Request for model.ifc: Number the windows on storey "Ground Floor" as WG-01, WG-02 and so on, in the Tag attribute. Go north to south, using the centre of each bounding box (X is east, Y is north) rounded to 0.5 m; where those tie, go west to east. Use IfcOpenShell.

First a look at what the model holds.

```python
import ifcopenshell
import ifcopenshell.util.element
import ifcopenshell.util.placement

model = ifcopenshell.open("model.ifc")
print(model.schema)
storey = next(s for s in model.by_type("IfcBuildingStorey") if s.Name == "Ground Floor")
windows = [e for e in ifcopenshell.util.element.get_decomposition(storey) if e.is_a("IfcWindow")]
for e in sorted(windows, key=lambda e: e.id()):
    origin = ifcopenshell.util.placement.get_local_placement(e.ObjectPlacement)[:3, 3]
    print(e.id(), e.Tag, e.Name, origin.round(2) + 0.0, sep=" | ")
```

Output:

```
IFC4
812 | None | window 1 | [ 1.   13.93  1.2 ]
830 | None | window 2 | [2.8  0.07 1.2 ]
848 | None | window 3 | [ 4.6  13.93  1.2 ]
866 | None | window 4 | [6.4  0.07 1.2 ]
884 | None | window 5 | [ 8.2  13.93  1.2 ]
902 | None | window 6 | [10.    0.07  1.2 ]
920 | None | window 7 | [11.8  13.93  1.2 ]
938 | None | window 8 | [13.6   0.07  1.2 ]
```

```python
import ifcopenshell
import ifcopenshell.geom
import ifcopenshell.util.element
import ifcopenshell.util.shape

model = ifcopenshell.open("model.ifc")
settings = ifcopenshell.geom.settings()
settings.set("use-world-coords", True)


def centre(element):
    shape = ifcopenshell.geom.create_shape(settings, element)
    return ifcopenshell.util.shape.get_bbox_centroid(shape.geometry)


storey = next(s for s in model.by_type("IfcBuildingStorey") if s.Name == "Ground Floor")
windows = [e for e in ifcopenshell.util.element.get_decomposition(storey) if e.is_a("IfcWindow")]

# Insertion points can sit at a corner or the storey origin, so sort by the geometry (in metres).
centres = {e: centre(e) for e in windows}
windows.sort(key=lambda e: (-round(centres[e][1] / 0.5), centres[e][0]))

for i, e in enumerate(windows, start=1):
    number = f"WG-{i:02d}"
    e.Tag = number
    print(e.id(), number)

model.write("model_updated.ifc")
```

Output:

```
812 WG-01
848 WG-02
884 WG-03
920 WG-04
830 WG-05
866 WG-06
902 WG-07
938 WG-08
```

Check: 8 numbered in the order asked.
